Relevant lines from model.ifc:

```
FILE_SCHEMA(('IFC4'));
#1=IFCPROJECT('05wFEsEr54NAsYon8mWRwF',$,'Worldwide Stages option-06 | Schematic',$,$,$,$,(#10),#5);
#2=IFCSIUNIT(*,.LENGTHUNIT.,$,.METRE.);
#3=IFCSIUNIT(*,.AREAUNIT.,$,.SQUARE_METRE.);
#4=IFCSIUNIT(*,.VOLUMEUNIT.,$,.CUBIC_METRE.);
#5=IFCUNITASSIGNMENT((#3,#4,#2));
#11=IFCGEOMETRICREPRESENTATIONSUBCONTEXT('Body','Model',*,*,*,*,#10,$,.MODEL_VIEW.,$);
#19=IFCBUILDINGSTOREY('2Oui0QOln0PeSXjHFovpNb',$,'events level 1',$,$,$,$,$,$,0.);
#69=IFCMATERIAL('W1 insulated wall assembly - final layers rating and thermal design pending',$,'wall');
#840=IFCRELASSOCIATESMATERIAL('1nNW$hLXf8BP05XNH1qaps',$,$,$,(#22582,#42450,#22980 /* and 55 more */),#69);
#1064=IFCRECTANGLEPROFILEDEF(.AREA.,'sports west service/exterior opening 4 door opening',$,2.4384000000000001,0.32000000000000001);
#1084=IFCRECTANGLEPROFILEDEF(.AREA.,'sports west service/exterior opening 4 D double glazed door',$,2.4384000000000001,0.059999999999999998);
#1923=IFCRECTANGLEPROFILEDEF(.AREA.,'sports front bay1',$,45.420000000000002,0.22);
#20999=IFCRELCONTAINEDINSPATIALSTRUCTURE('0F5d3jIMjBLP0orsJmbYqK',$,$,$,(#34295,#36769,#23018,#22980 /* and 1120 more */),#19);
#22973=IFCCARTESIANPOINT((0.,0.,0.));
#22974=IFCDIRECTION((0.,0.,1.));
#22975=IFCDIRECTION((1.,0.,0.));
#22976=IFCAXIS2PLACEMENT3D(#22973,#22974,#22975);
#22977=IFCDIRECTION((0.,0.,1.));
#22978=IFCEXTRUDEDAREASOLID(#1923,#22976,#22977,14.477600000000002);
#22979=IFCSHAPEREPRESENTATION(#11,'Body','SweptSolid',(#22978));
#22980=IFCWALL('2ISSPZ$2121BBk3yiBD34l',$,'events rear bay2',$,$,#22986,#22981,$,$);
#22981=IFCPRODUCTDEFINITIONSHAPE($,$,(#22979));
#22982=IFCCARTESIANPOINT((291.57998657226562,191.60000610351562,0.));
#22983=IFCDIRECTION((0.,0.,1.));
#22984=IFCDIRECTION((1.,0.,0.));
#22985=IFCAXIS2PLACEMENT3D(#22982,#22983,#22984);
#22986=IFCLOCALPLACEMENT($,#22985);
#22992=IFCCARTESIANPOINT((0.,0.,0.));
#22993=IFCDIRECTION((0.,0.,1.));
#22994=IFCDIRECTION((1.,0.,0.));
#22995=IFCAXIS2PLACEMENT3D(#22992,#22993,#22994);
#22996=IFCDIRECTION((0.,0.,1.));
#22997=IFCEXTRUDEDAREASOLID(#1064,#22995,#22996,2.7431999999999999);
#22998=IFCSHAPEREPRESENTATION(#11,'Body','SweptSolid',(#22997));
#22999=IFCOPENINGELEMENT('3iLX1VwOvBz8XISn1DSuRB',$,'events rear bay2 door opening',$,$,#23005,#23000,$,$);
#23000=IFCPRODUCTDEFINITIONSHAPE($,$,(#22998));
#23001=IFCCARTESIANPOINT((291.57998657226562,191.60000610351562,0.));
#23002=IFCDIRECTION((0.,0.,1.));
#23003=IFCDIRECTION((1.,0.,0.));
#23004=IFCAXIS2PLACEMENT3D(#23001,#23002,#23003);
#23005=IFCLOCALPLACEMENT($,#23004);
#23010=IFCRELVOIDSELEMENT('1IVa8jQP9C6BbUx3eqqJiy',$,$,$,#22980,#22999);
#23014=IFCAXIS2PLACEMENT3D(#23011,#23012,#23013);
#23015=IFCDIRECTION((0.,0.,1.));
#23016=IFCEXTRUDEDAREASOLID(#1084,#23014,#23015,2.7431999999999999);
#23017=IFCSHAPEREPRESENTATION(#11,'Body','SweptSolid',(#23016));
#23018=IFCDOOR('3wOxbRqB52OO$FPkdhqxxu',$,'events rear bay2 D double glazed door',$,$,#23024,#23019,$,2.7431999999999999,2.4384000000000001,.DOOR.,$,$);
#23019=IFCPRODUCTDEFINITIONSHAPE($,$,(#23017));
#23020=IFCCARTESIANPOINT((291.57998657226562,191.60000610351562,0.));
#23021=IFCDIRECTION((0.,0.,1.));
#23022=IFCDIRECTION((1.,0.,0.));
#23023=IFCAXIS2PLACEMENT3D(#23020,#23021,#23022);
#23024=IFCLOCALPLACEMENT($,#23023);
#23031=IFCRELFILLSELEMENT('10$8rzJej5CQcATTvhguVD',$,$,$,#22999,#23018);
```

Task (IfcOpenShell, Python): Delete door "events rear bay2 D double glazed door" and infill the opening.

```python
import ifcopenshell
import ifcopenshell.api.feature
import ifcopenshell.api.root
import ifcopenshell.geom
import ifcopenshell.util.shape

model = ifcopenshell.open("model.ifc")
settings = ifcopenshell.geom.settings()


def volume(element):
    """Net volume in cubic metres, openings subtracted."""
    shape = ifcopenshell.geom.create_shape(settings, element)
    return ifcopenshell.util.shape.get_volume(shape.geometry)


door = model.by_id(23018)
opening = door.FillsVoids[0].RelatingOpeningElement
wall = opening.VoidsElements[0].RelatingBuildingElement
before = volume(wall)

ifcopenshell.api.root.remove_product(model, product=door)
ifcopenshell.api.feature.remove_feature(model, feature=opening)

after = volume(wall)

print(f"wall volume {before:.3f} -> {after:.3f} m3")

model.write("model_edited.ifc")
```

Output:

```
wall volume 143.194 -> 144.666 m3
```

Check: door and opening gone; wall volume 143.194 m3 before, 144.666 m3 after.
